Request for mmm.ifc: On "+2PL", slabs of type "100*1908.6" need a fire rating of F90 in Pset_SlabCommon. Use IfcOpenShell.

First a look at what the model holds.

```python
import ifcopenshell
import ifcopenshell.util.element

model = ifcopenshell.open("mmm.ifc")
print(model.schema)
storey = next(s for s in model.by_type("IfcBuildingStorey") if s.Name == "+2PL")
slabs = [e for e in ifcopenshell.util.element.get_decomposition(storey) if e.is_a("IfcSlab")]
seen = {}
for e in slabs:
    element_type = ifcopenshell.util.element.get_type(e)
    key = (element_type.Name if element_type != e and element_type else None, ifcopenshell.util.element.get_pset(e, "Pset_SlabCommon", "FireRating"))
    seen[key] = seen.get(key, 0) + 1
for (name, value), count in sorted(seen.items(), key=str):
    print(count, "x", name, "|", value)
```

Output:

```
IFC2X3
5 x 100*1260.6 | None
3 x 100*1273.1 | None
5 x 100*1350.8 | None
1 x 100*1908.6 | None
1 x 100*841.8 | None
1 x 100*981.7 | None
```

```python
import ifcopenshell
import ifcopenshell.api.pset
import ifcopenshell.util.element

model = ifcopenshell.open("mmm.ifc")

storey = next(s for s in model.by_type("IfcBuildingStorey") if s.Name == "+2PL")
slabs = [e for e in ifcopenshell.util.element.get_decomposition(storey) if e.is_a("IfcSlab")]

count = 0
for e in slabs:
    element_type = ifcopenshell.util.element.get_type(e)
    if element_type in (None, e) or element_type.Name != "100*1908.6":
        continue
    found = ifcopenshell.util.element.get_pset(e, "Pset_SlabCommon", should_inherit=False)
    if found:
        pset = model.by_id(found["id"])
        if len(ifcopenshell.util.element.get_elements_by_pset(pset)) > 1:
            pset = ifcopenshell.api.pset.unshare_pset(model, products=[e], pset=pset)[0]
    else:
        pset = ifcopenshell.api.pset.add_pset(model, product=e, name="Pset_SlabCommon")
    ifcopenshell.api.pset.edit_pset(model, pset=pset, properties={"FireRating": "F90"})
    count += 1

print(count, "slabs updated")

model.write("mmm_rev.ifc")
```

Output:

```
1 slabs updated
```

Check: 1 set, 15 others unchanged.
